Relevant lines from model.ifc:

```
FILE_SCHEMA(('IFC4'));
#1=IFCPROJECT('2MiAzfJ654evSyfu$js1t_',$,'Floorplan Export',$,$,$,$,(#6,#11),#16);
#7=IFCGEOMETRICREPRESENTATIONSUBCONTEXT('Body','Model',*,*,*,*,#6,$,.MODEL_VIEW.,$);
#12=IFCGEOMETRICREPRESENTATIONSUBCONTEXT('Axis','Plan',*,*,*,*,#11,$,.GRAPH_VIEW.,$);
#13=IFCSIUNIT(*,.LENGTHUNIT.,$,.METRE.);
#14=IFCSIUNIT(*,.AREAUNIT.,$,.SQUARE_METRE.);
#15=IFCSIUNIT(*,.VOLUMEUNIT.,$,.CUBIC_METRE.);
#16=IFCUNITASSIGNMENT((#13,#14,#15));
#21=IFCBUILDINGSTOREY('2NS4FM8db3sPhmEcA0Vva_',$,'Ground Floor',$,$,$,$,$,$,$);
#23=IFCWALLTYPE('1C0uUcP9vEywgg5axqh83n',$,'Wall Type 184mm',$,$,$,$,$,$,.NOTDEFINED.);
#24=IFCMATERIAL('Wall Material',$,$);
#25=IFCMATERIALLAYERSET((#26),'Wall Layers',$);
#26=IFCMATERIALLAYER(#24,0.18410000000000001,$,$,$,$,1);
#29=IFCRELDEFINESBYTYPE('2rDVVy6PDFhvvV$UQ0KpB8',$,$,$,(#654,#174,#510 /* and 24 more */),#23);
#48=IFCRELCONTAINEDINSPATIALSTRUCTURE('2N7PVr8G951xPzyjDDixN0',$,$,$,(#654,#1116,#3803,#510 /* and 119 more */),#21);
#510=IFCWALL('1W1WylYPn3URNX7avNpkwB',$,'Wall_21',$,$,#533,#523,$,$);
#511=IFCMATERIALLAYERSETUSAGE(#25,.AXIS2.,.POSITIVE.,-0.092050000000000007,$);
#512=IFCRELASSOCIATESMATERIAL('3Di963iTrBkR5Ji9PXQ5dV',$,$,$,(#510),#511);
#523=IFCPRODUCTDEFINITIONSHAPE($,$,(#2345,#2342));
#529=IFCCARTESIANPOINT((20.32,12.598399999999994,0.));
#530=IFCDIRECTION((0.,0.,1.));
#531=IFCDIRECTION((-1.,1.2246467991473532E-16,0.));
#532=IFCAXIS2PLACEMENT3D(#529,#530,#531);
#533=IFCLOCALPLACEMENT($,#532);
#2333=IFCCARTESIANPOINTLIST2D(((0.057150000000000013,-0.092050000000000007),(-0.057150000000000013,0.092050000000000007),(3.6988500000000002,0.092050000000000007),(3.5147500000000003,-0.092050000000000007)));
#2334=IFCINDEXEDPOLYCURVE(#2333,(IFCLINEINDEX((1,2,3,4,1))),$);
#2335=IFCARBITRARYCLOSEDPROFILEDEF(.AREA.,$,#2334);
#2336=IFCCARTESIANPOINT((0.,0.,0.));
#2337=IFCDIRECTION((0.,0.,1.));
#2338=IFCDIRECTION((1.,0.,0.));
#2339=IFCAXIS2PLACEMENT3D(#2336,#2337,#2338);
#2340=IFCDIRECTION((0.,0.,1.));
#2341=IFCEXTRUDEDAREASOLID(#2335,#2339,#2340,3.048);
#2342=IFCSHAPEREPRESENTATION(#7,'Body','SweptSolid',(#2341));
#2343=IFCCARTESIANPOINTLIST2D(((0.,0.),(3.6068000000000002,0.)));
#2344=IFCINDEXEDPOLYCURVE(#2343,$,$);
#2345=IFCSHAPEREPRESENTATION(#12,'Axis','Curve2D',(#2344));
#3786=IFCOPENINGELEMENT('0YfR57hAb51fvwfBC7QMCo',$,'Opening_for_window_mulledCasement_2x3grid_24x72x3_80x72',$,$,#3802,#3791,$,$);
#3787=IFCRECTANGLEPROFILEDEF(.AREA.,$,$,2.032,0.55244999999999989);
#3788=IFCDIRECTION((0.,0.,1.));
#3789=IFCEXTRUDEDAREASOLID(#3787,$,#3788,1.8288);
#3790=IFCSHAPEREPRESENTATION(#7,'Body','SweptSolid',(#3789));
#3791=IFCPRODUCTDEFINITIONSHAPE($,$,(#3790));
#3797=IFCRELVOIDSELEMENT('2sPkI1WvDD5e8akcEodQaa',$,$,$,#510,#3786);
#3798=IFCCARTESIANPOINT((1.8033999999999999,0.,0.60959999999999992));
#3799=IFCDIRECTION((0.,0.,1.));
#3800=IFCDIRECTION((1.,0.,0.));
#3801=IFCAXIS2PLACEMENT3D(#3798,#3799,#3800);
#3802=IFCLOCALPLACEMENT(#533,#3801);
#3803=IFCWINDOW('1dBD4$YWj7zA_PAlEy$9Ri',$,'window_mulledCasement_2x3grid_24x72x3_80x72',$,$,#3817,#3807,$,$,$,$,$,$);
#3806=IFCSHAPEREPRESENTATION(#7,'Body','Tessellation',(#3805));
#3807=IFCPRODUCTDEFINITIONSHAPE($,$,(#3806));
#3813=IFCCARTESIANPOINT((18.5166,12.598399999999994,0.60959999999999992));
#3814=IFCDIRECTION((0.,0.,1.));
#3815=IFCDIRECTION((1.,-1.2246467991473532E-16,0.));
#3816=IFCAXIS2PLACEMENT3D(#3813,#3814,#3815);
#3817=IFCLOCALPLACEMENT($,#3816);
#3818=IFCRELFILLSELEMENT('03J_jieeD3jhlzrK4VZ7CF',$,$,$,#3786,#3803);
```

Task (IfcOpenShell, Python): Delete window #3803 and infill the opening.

```python
import ifcopenshell
import ifcopenshell.api.feature
import ifcopenshell.api.root
import ifcopenshell.geom
import ifcopenshell.util.shape

model = ifcopenshell.open("model.ifc")
settings = ifcopenshell.geom.settings()


def volume(element):
    """Net volume in cubic metres, openings subtracted."""
    shape = ifcopenshell.geom.create_shape(settings, element)
    return ifcopenshell.util.shape.get_volume(shape.geometry)


window = model.by_id(3803)
opening = window.FillsVoids[0].RelatingOpeningElement
wall = opening.VoidsElements[0].RelatingBuildingElement
before = volume(wall)

ifcopenshell.api.root.remove_product(model, product=window)
ifcopenshell.api.feature.remove_feature(model, feature=opening)

after = volume(wall)

print(f"wall volume {before:.3f} -> {after:.3f} m3")

model.write("model_rev.ifc")
```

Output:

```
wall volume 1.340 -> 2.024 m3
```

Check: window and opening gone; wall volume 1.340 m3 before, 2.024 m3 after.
